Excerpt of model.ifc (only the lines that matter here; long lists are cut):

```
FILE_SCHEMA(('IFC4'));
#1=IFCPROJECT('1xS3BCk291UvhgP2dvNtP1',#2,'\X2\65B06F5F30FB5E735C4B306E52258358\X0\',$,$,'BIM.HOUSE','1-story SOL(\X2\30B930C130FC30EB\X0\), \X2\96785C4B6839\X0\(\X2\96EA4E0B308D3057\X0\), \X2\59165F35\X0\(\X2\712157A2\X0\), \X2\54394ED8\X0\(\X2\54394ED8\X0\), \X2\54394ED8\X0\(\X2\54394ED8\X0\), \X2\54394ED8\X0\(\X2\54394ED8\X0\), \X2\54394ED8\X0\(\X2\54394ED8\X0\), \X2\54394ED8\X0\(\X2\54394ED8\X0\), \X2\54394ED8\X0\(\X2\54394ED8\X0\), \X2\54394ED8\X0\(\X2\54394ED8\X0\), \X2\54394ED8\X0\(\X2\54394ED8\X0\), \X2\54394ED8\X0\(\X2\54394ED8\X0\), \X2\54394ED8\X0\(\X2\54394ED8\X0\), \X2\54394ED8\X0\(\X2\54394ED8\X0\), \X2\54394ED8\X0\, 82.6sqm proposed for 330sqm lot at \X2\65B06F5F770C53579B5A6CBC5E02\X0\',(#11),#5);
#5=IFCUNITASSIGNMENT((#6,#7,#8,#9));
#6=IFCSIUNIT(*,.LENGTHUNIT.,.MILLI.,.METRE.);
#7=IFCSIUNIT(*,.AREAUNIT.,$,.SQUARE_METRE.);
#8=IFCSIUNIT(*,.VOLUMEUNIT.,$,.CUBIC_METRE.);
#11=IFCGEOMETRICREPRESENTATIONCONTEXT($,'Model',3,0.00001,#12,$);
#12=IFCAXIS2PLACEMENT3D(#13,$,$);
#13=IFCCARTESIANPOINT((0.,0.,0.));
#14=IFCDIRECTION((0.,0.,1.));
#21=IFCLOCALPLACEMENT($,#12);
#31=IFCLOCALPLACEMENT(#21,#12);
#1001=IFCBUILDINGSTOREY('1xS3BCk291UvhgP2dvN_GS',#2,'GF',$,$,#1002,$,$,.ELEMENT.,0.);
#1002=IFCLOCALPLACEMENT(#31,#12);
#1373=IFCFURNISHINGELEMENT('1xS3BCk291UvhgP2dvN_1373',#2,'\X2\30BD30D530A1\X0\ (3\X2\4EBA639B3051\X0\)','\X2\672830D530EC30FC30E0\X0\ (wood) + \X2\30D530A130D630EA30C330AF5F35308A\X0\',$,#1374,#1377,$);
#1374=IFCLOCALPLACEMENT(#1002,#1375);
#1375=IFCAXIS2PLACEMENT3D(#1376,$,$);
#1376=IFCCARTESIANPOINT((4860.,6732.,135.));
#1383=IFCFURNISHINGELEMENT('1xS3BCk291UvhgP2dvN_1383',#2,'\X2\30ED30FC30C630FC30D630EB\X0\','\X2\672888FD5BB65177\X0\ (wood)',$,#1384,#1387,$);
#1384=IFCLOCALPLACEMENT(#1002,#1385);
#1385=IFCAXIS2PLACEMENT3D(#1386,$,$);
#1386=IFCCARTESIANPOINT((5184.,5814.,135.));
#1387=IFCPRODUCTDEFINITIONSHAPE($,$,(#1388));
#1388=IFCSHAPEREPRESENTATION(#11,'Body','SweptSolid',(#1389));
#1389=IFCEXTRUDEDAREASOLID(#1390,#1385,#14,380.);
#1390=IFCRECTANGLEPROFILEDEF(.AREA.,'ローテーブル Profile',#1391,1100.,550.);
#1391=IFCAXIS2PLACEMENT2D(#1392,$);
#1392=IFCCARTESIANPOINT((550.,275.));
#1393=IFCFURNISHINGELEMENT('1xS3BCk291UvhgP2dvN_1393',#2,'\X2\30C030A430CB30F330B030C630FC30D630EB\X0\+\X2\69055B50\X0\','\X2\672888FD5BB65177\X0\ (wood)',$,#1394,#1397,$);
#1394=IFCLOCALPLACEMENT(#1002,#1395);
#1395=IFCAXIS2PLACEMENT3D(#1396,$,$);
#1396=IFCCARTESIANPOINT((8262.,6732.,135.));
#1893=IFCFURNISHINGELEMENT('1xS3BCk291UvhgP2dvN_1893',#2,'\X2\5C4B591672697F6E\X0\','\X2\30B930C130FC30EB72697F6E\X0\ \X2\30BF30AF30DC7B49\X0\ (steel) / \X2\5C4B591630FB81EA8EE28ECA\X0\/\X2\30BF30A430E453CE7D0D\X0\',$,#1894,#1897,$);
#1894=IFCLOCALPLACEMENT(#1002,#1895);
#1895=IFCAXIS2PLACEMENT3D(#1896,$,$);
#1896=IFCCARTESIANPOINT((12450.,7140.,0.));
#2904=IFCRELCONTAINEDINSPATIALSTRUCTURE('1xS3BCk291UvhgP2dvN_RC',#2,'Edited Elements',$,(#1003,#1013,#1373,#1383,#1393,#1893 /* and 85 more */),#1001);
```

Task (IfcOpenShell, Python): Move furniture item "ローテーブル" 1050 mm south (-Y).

```python
import ifcopenshell
import ifcopenshell.api.geometry
import ifcopenshell.util.placement

model = ifcopenshell.open("model.ifc")

item = model.by_guid("1xS3BCk291UvhgP2dvN_1383")
matrix = ifcopenshell.util.placement.get_local_placement(item.ObjectPlacement)
matrix[1, 3] -= 1050.0
ifcopenshell.api.geometry.edit_object_placement(model, product=item, matrix=matrix, is_si=False)

print(ifcopenshell.util.placement.get_local_placement(item.ObjectPlacement).round(3) + 0.0)

model.write("model_v2.ifc")
```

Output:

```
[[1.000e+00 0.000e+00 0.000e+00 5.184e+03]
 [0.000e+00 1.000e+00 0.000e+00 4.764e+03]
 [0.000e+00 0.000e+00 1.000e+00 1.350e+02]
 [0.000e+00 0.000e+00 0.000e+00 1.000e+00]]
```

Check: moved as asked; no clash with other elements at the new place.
